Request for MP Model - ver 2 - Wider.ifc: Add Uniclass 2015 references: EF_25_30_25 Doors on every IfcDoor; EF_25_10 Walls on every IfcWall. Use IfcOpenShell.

First a look at what the model holds.

```python
import ifcopenshell

model = ifcopenshell.open("MP Model - ver 2 - Wider.ifc")
print(model.schema)
print("classifications:", [c.Name for c in model.by_type("IfcClassification")])
for ifc_class in ("IfcDoor", "IfcRoof", "IfcStair", "IfcWall", "IfcWindow"):
    print(ifc_class, len(model.by_type(ifc_class)))
```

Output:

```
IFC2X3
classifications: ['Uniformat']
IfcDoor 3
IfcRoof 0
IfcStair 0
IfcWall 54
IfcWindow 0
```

```python
import ifcopenshell
import ifcopenshell.api.classification

model = ifcopenshell.open("MP Model - ver 2 - Wider.ifc")

# IFC2X3 requires Source and Edition and has no link from the project to the system.
system = model.create_entity("IfcClassification", Source="NBS", Edition="2015", Name="Uniclass 2015")

codes = {
    "IfcDoor": ("EF_25_30_25", "Doors"),
    "IfcWall": ("EF_25_10", "Walls"),
}
for ifc_class, (code, name) in codes.items():
    products = model.by_type(ifc_class)
    ifcopenshell.api.classification.add_reference(
        model, products=products, classification=system, identification=code, name=name
    )
    print(code, len(products))

model.write("MP Model - ver 2 - Wider_v2.ifc")
```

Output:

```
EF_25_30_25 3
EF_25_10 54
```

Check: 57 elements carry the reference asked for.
